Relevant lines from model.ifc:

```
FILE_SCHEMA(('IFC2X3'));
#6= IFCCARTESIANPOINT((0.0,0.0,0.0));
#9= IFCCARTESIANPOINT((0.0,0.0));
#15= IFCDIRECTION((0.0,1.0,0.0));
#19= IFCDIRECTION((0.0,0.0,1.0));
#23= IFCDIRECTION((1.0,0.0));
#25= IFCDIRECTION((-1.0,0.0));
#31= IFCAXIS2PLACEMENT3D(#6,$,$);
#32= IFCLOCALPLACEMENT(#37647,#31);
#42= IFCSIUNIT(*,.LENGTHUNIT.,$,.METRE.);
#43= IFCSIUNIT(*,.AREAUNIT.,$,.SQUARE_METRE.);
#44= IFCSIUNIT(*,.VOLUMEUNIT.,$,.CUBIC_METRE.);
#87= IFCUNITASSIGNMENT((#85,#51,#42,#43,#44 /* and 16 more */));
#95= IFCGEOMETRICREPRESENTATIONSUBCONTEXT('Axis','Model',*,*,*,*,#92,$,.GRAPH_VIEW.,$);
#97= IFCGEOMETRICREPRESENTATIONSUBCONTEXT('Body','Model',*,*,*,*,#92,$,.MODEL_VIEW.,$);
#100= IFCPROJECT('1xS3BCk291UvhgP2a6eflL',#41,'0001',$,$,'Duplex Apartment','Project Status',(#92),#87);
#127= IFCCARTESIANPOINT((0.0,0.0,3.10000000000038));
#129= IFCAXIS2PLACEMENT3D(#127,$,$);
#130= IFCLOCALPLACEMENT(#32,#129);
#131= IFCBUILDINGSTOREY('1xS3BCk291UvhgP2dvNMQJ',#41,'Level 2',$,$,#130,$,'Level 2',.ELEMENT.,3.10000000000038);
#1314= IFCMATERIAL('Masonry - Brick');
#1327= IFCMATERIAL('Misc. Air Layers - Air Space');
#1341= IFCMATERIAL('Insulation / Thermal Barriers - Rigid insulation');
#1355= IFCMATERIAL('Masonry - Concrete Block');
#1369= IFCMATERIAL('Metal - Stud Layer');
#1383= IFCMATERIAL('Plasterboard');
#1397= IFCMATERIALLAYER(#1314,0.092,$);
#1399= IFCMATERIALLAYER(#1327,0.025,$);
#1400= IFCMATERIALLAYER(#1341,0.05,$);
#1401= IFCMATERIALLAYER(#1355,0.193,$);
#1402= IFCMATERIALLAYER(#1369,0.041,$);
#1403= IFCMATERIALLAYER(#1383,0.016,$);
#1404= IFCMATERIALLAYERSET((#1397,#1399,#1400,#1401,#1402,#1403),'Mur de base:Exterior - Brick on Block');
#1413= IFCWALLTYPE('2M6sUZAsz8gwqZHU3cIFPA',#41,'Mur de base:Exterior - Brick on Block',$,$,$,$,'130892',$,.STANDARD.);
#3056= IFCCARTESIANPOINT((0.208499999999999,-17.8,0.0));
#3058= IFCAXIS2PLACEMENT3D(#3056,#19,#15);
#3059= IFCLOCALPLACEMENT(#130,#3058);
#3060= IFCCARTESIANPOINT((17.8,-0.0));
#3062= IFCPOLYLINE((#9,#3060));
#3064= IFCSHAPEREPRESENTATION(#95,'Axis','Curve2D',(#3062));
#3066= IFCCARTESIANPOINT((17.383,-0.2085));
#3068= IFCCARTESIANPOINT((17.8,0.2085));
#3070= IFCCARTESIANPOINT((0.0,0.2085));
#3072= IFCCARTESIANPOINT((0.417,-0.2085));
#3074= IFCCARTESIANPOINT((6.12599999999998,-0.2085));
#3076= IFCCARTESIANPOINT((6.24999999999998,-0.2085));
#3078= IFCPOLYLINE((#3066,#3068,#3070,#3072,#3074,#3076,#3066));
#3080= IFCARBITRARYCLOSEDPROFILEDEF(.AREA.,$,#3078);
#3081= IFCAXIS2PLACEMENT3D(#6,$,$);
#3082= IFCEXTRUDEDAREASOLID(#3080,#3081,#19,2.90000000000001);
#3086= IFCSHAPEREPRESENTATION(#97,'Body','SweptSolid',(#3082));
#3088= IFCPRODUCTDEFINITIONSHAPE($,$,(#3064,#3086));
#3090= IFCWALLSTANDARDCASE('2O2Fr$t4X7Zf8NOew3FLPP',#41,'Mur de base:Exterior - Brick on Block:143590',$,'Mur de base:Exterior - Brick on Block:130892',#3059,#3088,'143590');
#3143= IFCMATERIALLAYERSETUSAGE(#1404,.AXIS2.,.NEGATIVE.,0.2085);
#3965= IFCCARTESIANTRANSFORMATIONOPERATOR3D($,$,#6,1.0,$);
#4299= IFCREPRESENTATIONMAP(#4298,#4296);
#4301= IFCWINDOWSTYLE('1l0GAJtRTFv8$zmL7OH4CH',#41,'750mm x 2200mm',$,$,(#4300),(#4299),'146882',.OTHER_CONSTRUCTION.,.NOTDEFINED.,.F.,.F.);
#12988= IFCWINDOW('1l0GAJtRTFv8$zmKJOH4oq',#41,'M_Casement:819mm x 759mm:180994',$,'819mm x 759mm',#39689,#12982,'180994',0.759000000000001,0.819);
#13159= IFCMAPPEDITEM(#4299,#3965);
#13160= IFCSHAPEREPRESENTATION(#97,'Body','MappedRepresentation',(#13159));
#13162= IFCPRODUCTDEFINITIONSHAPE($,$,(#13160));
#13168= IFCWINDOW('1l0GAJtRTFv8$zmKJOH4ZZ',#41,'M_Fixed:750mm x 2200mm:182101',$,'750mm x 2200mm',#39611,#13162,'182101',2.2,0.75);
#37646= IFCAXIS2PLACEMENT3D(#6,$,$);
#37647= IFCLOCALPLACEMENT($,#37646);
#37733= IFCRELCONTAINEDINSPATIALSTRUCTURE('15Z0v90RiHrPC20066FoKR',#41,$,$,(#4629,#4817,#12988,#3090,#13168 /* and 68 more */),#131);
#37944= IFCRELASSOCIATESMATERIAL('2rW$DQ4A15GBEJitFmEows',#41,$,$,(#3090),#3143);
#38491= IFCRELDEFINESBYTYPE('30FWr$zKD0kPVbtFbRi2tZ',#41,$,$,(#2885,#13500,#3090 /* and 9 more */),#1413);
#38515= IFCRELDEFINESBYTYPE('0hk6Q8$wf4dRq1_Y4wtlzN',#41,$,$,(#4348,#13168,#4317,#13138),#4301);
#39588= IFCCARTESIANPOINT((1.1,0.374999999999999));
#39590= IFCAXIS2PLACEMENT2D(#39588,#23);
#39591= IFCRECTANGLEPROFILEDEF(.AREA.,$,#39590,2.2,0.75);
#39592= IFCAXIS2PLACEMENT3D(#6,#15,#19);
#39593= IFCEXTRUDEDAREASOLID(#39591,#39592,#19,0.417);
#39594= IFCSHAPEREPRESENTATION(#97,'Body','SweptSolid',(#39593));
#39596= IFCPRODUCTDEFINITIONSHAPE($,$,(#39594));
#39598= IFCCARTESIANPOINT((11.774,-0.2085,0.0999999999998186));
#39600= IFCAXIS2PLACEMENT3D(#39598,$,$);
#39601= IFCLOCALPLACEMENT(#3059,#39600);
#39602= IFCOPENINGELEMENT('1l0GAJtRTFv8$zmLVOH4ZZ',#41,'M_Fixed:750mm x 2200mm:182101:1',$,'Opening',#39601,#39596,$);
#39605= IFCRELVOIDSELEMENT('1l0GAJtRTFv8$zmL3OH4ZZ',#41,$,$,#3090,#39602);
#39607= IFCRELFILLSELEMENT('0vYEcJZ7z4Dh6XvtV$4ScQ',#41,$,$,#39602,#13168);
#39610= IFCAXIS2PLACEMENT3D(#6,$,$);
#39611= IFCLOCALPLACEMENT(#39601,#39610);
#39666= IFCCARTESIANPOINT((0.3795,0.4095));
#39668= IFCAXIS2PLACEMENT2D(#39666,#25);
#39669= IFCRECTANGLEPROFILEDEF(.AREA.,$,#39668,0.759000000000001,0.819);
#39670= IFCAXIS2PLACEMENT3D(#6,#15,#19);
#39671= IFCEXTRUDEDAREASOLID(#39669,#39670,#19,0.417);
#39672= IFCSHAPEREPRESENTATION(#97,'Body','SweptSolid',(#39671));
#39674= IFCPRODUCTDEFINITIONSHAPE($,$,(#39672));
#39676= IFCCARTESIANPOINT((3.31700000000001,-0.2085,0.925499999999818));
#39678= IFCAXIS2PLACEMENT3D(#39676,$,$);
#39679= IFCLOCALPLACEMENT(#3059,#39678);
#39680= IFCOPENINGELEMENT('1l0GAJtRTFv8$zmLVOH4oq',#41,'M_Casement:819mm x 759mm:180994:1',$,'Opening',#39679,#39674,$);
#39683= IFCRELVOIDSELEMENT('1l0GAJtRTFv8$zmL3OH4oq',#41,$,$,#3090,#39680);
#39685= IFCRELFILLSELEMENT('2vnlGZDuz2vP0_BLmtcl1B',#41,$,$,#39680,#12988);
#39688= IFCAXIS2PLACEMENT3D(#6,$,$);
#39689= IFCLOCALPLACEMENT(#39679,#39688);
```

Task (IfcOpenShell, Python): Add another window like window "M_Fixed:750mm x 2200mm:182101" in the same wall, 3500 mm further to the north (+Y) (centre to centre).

```python
import ifcopenshell
import ifcopenshell.api.feature
import ifcopenshell.api.geometry
import ifcopenshell.api.root
import ifcopenshell.geom
import ifcopenshell.util.element
import ifcopenshell.util.placement
import ifcopenshell.util.shape
import ifcopenshell.util.unit

model = ifcopenshell.open("model.ifc")
unit_scale = ifcopenshell.util.unit.calculate_unit_scale(model)
settings = ifcopenshell.geom.settings()


def volume(element):
    """Net volume in cubic metres, openings subtracted."""
    shape = ifcopenshell.geom.create_shape(settings, element)
    return ifcopenshell.util.shape.get_volume(shape.geometry)


def reuse_history(source, copy):
    """copy_class also copies each property set's owner history, people and application; keep the originals."""
    for rel in copy.IsDefinedBy:
        if rel.is_a("IfcRelDefinesByProperties") and (history := rel.RelatingPropertyDefinition.OwnerHistory):
            rel.RelatingPropertyDefinition.OwnerHistory = source.OwnerHistory
            ifcopenshell.util.element.remove_deep2(model, history)


window = model.by_guid("1l0GAJtRTFv8$zmKJOH4ZZ")
opening = window.FillsVoids[0].RelatingOpeningElement
wall = opening.VoidsElements[0].RelatingBuildingElement
before = volume(wall)
shift = ifcopenshell.util.placement.get_local_placement(wall.ObjectPlacement)[:3, 0] * 3.5 / unit_scale

# copy_class copies the void relationship, type, container and properties, but no geometry.
new_opening = ifcopenshell.api.root.copy_class(model, product=opening)
new_opening.Representation = ifcopenshell.util.element.copy_deep(
    model, opening.Representation, exclude=["IfcGeometricRepresentationContext", "IfcRepresentationMap"]
)
new_opening.Name = "M_Fixed:750mm x 2200mm"
new_window = ifcopenshell.api.root.copy_class(model, product=window)
new_window.Representation = ifcopenshell.util.element.copy_deep(
    model, window.Representation, exclude=["IfcGeometricRepresentationContext", "IfcRepresentationMap"]
)
new_window.Name = "M_Fixed:750mm x 2200mm"
new_window.Tag = None
reuse_history(window, new_window)
fills = ifcopenshell.api.feature.add_filling(model, opening=new_opening, element=new_window)
fills.OwnerHistory = new_window.OwnerHistory  # required in IFC2X3

for old, new in ((opening, new_opening), (window, new_window)):
    matrix = ifcopenshell.util.placement.get_local_placement(old.ObjectPlacement)
    matrix[:3, 3] += shift
    ifcopenshell.api.geometry.edit_object_placement(model, product=new, matrix=matrix, is_si=False)

after = volume(wall)

print(f"wall volume {before:.3f} -> {after:.3f} m3")

model.write("model-out.ifc")
```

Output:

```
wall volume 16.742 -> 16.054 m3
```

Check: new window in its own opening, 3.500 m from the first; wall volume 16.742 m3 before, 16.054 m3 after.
